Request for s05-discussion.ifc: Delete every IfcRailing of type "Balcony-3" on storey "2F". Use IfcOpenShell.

First a look at what the model holds.

```python
import ifcopenshell
import ifcopenshell.util.element

model = ifcopenshell.open("s05-discussion.ifc")
print(model.schema)
storey = next(s for s in model.by_type("IfcBuildingStorey") if s.Name == "2F")
railings = [e for e in ifcopenshell.util.element.get_decomposition(storey) if e.is_a("IfcRailing")]
seen = {}
for e in railings:
    element_type = ifcopenshell.util.element.get_type(e)
    name = element_type.Name if element_type not in (None, e) else None
    seen[name] = seen.get(name, 0) + 1
for name, count in sorted(seen.items(), key=str):
    print(count, "x", name)
```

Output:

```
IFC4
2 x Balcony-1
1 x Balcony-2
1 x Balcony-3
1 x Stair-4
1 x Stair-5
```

```python
import ifcopenshell
import ifcopenshell.api.root
import ifcopenshell.util.element

model = ifcopenshell.open("s05-discussion.ifc")

storey = next(s for s in model.by_type("IfcBuildingStorey") if s.Name == "2F")
railings = [e for e in ifcopenshell.util.element.get_decomposition(storey) if e.is_a("IfcRailing")]
targets = [e for e in railings if (t := ifcopenshell.util.element.get_type(e)) not in (None, e) and t.Name == "Balcony-3"]

for e in targets:
    ifcopenshell.api.root.remove_product(model, product=e)
print(len(targets), "removed")

model.write("s05-discussion_v2.ifc")
```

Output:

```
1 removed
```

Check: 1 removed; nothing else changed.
